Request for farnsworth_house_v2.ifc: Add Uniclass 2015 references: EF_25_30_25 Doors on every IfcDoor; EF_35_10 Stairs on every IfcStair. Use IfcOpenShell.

First a look at what the model holds.

```python
import ifcopenshell

model = ifcopenshell.open("farnsworth_house_v2.ifc")
print(model.schema)
print("classifications:", [c.Name for c in model.by_type("IfcClassification")])
for ifc_class in ("IfcDoor", "IfcRoof", "IfcStair", "IfcWall", "IfcWindow"):
    print(ifc_class, len(model.by_type(ifc_class)))
```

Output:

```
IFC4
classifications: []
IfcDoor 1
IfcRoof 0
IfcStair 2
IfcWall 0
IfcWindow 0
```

```python
import ifcopenshell
import ifcopenshell.api.classification

model = ifcopenshell.open("farnsworth_house_v2.ifc")

system = ifcopenshell.api.classification.add_classification(model, classification="Uniclass 2015")

codes = {
    "IfcDoor": ("EF_25_30_25", "Doors"),
    "IfcStair": ("EF_35_10", "Stairs"),
}
for ifc_class, (code, name) in codes.items():
    products = model.by_type(ifc_class)
    ifcopenshell.api.classification.add_reference(
        model, products=products, classification=system, identification=code, name=name
    )
    print(code, len(products))

model.write("farnsworth_house_v2-out.ifc")
```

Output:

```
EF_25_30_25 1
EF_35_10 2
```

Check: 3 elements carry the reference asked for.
